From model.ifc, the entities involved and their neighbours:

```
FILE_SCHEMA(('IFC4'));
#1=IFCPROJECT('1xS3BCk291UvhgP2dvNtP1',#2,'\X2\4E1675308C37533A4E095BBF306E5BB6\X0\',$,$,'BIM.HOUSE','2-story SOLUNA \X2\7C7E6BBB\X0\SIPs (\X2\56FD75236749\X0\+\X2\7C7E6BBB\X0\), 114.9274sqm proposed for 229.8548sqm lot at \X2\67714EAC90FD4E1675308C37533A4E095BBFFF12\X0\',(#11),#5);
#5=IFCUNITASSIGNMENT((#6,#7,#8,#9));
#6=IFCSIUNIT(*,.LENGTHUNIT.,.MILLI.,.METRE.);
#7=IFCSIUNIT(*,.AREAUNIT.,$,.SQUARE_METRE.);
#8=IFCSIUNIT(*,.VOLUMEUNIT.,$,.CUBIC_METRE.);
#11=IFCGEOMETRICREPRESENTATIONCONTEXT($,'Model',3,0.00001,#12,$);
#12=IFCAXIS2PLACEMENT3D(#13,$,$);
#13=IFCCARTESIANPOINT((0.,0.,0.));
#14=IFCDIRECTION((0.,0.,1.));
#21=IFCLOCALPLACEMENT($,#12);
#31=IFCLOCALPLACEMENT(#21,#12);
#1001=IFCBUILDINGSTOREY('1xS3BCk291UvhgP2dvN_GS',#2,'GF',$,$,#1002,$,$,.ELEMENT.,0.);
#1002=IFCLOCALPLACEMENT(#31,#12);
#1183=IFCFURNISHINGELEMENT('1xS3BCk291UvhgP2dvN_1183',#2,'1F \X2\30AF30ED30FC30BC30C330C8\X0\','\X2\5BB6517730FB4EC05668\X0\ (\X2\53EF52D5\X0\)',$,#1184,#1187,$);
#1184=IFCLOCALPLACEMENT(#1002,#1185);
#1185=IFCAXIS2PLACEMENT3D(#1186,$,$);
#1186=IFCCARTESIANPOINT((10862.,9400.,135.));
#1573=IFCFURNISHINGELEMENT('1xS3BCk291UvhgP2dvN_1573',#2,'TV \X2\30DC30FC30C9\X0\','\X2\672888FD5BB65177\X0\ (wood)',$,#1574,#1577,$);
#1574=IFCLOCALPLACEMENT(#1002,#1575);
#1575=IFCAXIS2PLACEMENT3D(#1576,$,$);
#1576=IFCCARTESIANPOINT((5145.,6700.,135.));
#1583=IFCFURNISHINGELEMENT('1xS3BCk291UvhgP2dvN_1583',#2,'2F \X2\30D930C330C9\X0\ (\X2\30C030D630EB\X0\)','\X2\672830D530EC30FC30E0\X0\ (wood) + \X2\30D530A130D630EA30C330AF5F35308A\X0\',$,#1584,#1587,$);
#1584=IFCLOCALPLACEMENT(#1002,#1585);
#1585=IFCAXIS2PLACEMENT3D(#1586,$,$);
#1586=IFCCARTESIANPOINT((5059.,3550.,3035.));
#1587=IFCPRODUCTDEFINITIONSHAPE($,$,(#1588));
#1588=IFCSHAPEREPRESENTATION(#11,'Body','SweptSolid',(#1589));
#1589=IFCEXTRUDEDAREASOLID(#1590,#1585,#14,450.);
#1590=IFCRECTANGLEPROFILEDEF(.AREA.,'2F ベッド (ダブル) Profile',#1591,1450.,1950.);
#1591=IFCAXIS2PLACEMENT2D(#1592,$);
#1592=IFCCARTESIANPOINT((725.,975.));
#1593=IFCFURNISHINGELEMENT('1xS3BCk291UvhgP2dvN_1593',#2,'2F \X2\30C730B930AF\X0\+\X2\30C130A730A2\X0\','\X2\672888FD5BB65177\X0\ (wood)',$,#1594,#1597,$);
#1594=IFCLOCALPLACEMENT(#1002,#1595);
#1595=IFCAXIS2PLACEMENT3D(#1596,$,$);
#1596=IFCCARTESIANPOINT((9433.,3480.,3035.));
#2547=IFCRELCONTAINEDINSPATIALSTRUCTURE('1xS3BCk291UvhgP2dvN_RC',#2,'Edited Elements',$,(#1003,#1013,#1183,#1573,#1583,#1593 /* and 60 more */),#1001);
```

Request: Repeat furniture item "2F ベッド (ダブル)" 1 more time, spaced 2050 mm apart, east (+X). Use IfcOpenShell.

```python
import numpy as np
import ifcopenshell
import ifcopenshell.api.geometry
import ifcopenshell.api.root
import ifcopenshell.util.element
import ifcopenshell.util.placement

model = ifcopenshell.open("model.ifc")


def reuse_history(source, copy):
    """copy_class also copies each property set's owner history, people and application; keep the originals."""
    for rel in copy.IsDefinedBy:
        if rel.is_a("IfcRelDefinesByProperties") and (history := rel.RelatingPropertyDefinition.OwnerHistory):
            rel.RelatingPropertyDefinition.OwnerHistory = source.OwnerHistory
            ifcopenshell.util.element.remove_deep2(model, history)


source = model.by_guid("1xS3BCk291UvhgP2dvN_1583")
base = ifcopenshell.util.placement.get_local_placement(source.ObjectPlacement)
step = np.array([1.0, 0.0, 0.0]) * 2050.0

for i in range(1, 2):
    copy = ifcopenshell.api.root.copy_class(model, product=source)
    copy.Representation = ifcopenshell.util.element.copy_deep(
        model, source.Representation, exclude=["IfcGeometricRepresentationContext", "IfcRepresentationMap"]
    )
    reuse_history(source, copy)
    matrix = base.copy()
    matrix[:3, 3] += i * step
    print("added at", matrix[:3, 3].round(3) + 0.0)
    ifcopenshell.api.geometry.edit_object_placement(model, product=copy, matrix=matrix, is_si=False)

model.write("model_updated.ifc")
```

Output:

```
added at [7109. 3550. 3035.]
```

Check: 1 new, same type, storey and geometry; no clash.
